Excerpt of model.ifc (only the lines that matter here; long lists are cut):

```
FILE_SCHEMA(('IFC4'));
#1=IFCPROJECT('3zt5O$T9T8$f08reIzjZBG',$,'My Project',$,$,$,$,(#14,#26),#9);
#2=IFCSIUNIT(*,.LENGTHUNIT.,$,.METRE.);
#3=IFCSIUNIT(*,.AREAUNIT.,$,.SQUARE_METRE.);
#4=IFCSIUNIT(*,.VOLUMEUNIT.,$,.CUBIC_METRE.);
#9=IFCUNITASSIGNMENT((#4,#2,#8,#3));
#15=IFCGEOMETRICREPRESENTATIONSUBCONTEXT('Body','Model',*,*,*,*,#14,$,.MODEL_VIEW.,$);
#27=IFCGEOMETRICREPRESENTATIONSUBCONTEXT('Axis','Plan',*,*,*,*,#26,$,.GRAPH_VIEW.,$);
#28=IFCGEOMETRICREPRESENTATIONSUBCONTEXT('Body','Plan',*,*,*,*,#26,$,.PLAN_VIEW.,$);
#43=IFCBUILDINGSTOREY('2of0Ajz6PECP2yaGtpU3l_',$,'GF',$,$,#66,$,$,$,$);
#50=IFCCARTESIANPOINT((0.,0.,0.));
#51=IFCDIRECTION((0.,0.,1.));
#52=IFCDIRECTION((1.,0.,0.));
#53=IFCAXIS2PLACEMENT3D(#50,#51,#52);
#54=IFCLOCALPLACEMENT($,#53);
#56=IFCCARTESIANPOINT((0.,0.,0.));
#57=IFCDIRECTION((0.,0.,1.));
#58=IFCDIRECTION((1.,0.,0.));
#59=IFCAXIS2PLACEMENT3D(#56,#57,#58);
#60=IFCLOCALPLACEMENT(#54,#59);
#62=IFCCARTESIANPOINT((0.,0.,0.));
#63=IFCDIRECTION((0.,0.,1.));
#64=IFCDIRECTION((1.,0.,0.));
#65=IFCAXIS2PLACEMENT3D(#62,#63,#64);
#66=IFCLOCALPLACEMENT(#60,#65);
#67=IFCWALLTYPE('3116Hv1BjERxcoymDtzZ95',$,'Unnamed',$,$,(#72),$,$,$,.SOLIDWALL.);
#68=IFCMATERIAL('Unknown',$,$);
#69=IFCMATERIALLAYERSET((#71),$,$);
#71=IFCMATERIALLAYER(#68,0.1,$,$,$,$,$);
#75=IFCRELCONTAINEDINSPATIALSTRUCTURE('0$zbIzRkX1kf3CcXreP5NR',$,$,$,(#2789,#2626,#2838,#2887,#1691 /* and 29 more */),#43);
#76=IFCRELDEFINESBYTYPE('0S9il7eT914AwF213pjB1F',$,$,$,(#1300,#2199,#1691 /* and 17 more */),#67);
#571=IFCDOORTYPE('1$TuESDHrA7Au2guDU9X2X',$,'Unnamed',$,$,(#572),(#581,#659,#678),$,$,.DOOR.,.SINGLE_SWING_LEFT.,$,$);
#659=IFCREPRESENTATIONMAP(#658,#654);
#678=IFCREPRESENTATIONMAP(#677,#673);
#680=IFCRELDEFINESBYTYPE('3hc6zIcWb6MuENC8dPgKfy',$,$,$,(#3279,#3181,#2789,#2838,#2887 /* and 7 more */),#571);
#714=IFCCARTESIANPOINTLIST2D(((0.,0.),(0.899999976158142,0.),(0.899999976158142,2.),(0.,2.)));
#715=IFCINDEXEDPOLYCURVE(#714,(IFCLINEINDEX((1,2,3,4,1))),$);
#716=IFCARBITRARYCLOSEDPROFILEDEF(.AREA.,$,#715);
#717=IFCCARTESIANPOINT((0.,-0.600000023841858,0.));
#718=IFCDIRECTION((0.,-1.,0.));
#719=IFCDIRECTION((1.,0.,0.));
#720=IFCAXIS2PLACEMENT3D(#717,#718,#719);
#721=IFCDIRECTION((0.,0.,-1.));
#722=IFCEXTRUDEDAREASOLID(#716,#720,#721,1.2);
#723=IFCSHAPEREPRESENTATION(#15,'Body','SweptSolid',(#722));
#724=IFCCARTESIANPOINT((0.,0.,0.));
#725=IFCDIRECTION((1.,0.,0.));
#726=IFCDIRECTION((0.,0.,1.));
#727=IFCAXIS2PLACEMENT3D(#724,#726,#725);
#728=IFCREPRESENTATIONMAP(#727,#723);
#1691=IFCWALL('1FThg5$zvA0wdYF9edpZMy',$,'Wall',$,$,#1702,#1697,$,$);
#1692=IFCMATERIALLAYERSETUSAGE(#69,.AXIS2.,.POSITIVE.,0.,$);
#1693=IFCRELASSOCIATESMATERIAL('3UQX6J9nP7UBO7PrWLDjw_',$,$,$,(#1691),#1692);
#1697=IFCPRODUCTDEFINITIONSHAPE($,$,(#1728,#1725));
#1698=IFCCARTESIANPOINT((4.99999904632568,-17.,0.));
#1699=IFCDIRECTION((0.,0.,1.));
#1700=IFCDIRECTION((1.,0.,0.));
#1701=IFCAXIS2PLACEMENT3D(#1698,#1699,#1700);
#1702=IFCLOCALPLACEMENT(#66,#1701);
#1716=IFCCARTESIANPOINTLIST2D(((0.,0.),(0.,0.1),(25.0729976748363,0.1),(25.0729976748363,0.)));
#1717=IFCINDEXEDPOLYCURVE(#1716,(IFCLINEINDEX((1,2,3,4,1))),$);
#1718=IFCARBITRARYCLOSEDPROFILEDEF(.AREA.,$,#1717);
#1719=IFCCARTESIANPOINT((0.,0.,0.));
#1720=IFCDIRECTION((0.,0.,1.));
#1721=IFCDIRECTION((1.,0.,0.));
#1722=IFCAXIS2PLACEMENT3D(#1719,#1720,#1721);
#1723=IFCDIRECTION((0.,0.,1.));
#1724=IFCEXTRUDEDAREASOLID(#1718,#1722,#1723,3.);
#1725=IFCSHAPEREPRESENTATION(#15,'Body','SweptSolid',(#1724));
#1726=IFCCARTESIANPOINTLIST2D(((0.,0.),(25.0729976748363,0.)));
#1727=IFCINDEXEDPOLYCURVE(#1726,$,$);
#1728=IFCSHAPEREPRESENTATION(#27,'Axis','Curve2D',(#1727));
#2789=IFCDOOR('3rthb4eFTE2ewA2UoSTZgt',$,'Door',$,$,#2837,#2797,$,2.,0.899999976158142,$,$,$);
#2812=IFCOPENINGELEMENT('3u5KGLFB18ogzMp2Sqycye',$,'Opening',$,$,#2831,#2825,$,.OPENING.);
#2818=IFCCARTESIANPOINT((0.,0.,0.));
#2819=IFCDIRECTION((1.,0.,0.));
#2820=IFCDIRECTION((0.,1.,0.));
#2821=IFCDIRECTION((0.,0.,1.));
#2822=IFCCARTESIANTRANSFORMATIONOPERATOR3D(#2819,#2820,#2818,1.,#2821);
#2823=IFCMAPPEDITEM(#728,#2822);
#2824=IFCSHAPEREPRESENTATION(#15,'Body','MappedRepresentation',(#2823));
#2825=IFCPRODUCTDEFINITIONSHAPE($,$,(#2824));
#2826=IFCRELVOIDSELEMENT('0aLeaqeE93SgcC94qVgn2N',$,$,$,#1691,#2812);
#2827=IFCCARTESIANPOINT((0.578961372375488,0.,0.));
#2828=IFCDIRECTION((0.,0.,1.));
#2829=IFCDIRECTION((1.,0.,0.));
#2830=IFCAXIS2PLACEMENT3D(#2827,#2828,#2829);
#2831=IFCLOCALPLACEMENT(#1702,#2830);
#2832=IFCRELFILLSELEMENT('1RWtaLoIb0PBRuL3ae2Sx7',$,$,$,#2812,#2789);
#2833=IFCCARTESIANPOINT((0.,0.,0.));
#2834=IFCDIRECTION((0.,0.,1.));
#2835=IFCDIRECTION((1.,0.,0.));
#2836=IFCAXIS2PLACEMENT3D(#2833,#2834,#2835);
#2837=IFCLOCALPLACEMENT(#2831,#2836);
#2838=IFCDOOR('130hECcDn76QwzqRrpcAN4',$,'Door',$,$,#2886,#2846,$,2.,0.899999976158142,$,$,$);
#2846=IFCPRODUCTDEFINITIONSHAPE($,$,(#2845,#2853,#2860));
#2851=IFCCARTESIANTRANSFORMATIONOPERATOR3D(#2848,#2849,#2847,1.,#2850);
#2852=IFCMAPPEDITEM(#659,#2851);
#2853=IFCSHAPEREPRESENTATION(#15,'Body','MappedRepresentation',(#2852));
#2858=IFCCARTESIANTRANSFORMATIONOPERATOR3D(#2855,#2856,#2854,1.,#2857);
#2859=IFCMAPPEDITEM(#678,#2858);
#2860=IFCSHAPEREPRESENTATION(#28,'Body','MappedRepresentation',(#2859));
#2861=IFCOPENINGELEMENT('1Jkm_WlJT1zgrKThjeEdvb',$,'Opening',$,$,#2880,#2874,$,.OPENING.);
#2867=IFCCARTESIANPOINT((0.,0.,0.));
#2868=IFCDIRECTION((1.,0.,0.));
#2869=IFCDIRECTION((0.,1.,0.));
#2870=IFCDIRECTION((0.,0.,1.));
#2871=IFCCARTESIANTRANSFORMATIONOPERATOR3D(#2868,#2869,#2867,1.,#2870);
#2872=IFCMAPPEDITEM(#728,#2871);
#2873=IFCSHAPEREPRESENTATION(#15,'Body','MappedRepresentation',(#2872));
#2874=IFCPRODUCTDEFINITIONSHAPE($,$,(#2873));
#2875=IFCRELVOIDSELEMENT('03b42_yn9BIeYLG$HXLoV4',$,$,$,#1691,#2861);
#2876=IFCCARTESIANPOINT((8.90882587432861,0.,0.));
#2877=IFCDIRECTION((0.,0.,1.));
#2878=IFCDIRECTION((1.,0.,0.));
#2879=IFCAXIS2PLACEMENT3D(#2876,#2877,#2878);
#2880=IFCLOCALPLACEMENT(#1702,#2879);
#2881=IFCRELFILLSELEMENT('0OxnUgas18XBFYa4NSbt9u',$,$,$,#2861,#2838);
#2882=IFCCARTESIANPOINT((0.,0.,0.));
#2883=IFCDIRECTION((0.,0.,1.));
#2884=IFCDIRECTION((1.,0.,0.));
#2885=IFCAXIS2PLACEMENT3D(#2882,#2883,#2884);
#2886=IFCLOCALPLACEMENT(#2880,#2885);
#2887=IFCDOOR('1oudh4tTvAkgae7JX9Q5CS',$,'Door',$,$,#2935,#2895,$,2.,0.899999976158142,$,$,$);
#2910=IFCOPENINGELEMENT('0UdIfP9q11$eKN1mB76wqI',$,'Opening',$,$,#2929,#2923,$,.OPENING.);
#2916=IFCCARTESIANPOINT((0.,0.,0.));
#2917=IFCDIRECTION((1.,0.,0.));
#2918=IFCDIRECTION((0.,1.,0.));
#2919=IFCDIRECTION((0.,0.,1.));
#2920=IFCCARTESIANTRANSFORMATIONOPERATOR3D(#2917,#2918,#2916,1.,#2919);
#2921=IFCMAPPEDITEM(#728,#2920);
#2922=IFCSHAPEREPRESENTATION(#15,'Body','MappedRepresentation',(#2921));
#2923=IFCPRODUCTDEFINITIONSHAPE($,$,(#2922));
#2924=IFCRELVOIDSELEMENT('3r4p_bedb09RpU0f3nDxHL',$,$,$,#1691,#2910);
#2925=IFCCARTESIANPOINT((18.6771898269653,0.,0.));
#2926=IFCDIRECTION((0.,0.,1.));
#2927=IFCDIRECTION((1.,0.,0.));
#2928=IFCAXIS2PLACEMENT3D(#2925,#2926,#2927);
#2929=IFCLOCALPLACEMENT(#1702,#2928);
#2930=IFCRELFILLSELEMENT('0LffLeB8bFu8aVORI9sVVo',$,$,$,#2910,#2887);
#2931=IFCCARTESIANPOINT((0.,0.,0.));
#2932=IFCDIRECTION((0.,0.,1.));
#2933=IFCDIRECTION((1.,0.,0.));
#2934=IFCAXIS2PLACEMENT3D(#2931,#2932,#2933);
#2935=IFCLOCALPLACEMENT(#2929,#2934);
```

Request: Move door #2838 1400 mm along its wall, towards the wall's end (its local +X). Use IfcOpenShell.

```python
import ifcopenshell
import ifcopenshell.api.geometry
import ifcopenshell.util.placement
import ifcopenshell.util.unit

model = ifcopenshell.open("model.ifc")
unit_scale = ifcopenshell.util.unit.calculate_unit_scale(model)

door = model.by_id(2838)
opening = door.FillsVoids[0].RelatingOpeningElement
wall = opening.VoidsElements[0].RelatingBuildingElement

wall_matrix = ifcopenshell.util.placement.get_local_placement(wall.ObjectPlacement)
shift = wall_matrix[:3, 0] * 1.4 / unit_scale
before = ifcopenshell.util.placement.get_local_placement(door.ObjectPlacement)[:3, 3].copy()

# The door is placed relative to its opening, so it follows when the opening moves.
matrix = ifcopenshell.util.placement.get_local_placement(opening.ObjectPlacement)
matrix[:3, 3] += shift
ifcopenshell.api.geometry.edit_object_placement(
    model, product=opening, matrix=matrix, is_si=False, should_transform_children=True
)

after = ifcopenshell.util.placement.get_local_placement(door.ObjectPlacement)[:3, 3]
print("door moved by", (after - before).round(3) + 0.0)

model.write("model_rev.ifc")
```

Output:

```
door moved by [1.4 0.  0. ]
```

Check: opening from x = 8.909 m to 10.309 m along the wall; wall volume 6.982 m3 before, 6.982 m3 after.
